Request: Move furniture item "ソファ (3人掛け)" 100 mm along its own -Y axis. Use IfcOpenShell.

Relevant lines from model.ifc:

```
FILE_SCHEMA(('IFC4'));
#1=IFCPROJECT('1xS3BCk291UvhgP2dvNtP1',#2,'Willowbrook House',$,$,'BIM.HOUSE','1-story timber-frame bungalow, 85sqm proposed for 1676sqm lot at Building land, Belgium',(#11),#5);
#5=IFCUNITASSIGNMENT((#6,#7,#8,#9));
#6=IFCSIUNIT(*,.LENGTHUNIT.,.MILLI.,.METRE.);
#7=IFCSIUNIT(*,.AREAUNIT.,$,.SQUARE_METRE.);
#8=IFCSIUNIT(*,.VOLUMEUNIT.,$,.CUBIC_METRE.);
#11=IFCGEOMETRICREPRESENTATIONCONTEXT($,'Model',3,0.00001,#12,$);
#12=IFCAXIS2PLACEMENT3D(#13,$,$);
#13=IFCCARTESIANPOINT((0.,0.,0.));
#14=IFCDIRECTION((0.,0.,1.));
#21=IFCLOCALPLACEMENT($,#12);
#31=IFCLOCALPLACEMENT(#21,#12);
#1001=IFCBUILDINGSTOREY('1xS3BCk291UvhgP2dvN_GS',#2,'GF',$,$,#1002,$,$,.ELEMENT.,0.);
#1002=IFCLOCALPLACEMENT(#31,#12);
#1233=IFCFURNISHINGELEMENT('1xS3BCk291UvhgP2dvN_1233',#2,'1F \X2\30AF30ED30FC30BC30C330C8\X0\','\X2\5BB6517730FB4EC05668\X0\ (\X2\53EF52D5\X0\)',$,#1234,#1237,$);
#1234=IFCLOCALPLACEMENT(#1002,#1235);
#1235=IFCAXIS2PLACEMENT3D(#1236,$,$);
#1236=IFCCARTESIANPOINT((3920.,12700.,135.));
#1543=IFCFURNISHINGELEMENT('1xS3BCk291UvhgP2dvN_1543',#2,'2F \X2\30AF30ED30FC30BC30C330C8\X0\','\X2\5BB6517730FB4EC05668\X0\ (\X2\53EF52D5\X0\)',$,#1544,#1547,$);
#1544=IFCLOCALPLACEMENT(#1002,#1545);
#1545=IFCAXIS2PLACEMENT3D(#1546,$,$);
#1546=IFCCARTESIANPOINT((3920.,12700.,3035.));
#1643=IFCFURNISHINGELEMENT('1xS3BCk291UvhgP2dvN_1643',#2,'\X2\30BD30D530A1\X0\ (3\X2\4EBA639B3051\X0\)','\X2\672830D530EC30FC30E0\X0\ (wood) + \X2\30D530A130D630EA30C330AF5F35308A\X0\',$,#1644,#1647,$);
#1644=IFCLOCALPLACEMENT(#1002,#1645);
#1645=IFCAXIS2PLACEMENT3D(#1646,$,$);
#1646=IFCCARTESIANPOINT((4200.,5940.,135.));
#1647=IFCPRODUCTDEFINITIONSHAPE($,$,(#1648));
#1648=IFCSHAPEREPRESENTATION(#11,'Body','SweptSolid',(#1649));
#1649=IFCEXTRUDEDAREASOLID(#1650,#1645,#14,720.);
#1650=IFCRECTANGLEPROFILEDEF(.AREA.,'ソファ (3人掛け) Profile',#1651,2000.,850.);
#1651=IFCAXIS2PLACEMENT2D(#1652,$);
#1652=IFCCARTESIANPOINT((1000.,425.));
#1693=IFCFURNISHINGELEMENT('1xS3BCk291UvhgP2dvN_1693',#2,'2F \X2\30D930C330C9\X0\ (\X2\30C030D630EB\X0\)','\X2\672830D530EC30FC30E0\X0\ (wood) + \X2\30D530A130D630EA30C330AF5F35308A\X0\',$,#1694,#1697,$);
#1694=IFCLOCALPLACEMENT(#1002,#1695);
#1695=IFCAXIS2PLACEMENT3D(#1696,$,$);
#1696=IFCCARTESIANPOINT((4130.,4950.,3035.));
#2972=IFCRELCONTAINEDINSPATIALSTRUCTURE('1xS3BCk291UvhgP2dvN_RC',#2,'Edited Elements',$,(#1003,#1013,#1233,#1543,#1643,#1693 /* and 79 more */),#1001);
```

```python
import ifcopenshell
import ifcopenshell.api.geometry
import ifcopenshell.util.placement

model = ifcopenshell.open("model.ifc")

item = model.by_guid("1xS3BCk291UvhgP2dvN_1643")
matrix = ifcopenshell.util.placement.get_local_placement(item.ObjectPlacement)
matrix[:3, 3] -= matrix[:3, 1] * 100.0
ifcopenshell.api.geometry.edit_object_placement(model, product=item, matrix=matrix, is_si=False)

print(ifcopenshell.util.placement.get_local_placement(item.ObjectPlacement).round(3) + 0.0)

model.write("model-out.ifc")
```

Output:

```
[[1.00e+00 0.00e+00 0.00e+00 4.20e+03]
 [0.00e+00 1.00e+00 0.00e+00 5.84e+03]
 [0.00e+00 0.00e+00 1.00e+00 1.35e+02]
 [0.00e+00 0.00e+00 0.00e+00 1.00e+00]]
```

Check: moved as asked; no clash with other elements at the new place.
